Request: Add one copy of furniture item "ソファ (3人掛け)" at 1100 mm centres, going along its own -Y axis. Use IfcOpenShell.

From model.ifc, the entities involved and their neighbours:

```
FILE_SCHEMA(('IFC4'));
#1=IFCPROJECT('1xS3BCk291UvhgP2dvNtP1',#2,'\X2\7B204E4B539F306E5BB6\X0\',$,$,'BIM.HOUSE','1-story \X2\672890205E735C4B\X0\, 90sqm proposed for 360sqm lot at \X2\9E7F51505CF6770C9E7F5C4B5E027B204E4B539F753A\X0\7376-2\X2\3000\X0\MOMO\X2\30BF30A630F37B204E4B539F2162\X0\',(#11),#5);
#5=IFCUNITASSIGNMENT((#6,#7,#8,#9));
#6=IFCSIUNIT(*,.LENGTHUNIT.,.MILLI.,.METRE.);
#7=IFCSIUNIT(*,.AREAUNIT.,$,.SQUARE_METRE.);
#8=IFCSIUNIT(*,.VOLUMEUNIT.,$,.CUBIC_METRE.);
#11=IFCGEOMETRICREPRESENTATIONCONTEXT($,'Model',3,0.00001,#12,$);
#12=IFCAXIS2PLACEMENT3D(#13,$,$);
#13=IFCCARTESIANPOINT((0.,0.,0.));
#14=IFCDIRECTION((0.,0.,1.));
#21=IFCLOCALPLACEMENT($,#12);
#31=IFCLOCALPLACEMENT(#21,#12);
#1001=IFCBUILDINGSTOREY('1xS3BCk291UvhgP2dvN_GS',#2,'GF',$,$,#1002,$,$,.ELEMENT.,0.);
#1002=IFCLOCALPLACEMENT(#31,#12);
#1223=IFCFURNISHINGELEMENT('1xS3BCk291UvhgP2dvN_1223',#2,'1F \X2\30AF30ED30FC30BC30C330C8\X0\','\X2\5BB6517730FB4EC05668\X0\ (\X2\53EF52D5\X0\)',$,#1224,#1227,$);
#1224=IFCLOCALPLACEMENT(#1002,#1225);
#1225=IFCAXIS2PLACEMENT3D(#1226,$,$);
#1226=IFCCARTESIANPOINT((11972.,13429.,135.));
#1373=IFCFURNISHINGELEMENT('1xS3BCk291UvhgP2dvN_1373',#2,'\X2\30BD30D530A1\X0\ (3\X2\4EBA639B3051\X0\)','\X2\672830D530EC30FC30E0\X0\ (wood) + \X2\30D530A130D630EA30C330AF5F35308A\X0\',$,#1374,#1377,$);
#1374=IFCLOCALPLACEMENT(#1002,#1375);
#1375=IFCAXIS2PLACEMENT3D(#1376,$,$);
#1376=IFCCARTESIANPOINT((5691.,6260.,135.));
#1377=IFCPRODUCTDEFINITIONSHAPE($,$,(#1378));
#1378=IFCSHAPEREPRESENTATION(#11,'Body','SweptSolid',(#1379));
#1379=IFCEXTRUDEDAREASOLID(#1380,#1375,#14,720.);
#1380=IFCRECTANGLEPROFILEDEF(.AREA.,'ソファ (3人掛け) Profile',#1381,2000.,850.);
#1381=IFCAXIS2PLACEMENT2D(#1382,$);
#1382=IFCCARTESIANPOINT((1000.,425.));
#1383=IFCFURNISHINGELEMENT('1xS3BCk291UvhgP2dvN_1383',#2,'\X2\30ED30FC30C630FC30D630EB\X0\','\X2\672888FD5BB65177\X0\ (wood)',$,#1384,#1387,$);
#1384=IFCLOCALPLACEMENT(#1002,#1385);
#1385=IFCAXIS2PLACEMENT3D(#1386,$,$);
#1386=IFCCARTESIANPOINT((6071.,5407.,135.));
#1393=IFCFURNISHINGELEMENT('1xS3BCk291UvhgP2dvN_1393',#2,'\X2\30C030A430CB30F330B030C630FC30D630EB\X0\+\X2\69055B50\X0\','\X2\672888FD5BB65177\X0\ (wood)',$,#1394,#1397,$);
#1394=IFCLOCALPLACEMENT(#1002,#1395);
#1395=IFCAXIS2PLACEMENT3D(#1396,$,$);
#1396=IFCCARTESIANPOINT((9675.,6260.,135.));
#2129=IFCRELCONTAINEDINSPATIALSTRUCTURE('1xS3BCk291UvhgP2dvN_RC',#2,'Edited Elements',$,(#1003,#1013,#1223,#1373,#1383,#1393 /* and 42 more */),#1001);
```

```python
import ifcopenshell
import ifcopenshell.api.geometry
import ifcopenshell.api.root
import ifcopenshell.util.element
import ifcopenshell.util.placement

model = ifcopenshell.open("model.ifc")


def reuse_history(source, copy):
    """copy_class also copies each property set's owner history, people and application; keep the originals."""
    for rel in copy.IsDefinedBy:
        if rel.is_a("IfcRelDefinesByProperties") and (history := rel.RelatingPropertyDefinition.OwnerHistory):
            rel.RelatingPropertyDefinition.OwnerHistory = source.OwnerHistory
            ifcopenshell.util.element.remove_deep2(model, history)


source = model.by_id(1373)
base = ifcopenshell.util.placement.get_local_placement(source.ObjectPlacement)
step = -base[:3, 1] * 1100.0

for i in range(1, 2):
    copy = ifcopenshell.api.root.copy_class(model, product=source)
    copy.Representation = ifcopenshell.util.element.copy_deep(
        model, source.Representation, exclude=["IfcGeometricRepresentationContext", "IfcRepresentationMap"]
    )
    reuse_history(source, copy)
    matrix = base.copy()
    matrix[:3, 3] += i * step
    print("added at", matrix[:3, 3].round(3) + 0.0)
    ifcopenshell.api.geometry.edit_object_placement(model, product=copy, matrix=matrix, is_si=False)

model.write("model_v2.ifc")
```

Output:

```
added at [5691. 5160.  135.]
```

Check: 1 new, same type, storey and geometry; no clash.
